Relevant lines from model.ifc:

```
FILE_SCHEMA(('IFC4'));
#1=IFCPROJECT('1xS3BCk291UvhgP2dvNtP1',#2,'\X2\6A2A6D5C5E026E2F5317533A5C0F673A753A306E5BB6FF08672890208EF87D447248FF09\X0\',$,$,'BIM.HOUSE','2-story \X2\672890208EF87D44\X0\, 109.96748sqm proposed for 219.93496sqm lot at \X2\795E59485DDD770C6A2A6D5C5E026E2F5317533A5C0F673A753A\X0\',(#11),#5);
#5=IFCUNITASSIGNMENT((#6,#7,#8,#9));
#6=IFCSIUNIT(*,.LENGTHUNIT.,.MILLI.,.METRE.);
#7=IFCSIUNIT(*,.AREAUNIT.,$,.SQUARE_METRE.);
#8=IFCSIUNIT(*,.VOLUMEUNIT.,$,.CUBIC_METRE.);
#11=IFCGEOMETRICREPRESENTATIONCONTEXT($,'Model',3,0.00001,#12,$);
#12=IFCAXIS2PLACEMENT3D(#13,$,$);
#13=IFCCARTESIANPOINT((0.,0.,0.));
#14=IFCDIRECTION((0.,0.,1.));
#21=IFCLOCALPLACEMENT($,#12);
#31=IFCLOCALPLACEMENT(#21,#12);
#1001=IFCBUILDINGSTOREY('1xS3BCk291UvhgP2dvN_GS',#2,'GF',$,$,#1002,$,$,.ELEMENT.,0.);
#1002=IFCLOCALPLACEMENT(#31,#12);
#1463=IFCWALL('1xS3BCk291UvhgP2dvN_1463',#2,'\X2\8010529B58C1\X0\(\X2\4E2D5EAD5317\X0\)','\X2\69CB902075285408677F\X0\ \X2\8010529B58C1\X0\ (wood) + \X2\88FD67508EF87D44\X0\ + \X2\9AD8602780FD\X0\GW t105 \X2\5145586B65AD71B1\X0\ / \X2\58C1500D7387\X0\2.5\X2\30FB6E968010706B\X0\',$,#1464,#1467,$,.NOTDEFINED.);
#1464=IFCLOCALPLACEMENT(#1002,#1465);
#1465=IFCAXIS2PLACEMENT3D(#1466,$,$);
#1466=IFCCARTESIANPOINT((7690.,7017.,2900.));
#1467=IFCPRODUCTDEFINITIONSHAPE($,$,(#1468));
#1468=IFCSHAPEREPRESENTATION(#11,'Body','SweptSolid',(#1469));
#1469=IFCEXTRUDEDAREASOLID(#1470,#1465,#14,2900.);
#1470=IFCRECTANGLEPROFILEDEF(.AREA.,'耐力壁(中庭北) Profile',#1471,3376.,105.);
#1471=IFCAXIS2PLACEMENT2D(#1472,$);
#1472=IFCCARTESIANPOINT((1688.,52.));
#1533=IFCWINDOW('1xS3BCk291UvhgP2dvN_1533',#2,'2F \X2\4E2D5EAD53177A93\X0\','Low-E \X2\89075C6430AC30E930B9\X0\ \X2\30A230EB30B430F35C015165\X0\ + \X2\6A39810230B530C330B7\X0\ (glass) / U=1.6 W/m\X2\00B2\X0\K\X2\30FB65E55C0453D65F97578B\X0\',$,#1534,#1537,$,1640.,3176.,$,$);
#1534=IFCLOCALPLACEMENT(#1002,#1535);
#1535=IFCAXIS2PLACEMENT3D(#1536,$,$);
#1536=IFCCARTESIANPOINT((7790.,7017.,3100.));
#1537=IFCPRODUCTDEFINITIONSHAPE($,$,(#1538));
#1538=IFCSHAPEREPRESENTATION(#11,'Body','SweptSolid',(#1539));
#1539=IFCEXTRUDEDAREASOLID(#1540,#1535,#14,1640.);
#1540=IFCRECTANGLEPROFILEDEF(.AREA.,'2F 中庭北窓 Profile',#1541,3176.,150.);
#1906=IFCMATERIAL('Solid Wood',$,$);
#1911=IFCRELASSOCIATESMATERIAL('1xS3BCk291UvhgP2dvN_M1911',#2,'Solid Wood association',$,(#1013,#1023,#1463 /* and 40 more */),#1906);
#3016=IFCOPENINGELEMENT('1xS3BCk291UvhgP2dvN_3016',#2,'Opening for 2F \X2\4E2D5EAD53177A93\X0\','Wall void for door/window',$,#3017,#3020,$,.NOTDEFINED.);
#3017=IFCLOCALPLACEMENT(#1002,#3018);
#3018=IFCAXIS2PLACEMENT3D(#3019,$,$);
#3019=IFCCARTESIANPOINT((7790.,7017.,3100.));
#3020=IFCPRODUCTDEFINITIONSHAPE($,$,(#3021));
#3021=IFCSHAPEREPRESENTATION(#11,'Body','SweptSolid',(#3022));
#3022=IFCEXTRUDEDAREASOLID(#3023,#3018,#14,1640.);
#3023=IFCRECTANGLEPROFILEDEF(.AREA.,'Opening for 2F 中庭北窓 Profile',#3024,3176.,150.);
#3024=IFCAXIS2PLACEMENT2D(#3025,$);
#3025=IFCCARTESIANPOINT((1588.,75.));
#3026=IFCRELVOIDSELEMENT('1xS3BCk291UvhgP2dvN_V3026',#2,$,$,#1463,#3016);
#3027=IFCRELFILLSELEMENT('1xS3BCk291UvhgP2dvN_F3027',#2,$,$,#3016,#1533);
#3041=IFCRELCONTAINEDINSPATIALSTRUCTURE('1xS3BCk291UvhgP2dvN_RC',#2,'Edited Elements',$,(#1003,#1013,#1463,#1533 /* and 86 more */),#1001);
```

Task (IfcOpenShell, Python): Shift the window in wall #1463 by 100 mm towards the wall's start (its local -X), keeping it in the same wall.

```python
import ifcopenshell
import ifcopenshell.api.geometry
import ifcopenshell.util.placement

model = ifcopenshell.open("model.ifc")

window = model.by_id(1533)
opening = window.FillsVoids[0].RelatingOpeningElement
wall = opening.VoidsElements[0].RelatingBuildingElement

wall_matrix = ifcopenshell.util.placement.get_local_placement(wall.ObjectPlacement)
shift = wall_matrix[:3, 0] * -100.0
before = ifcopenshell.util.placement.get_local_placement(window.ObjectPlacement)[:3, 3].copy()

# The window is not placed relative to its opening, so move both.
for product in (opening, window):
    matrix = ifcopenshell.util.placement.get_local_placement(product.ObjectPlacement)
    matrix[:3, 3] += shift
    ifcopenshell.api.geometry.edit_object_placement(model, product=product, matrix=matrix, is_si=False)

after = ifcopenshell.util.placement.get_local_placement(window.ObjectPlacement)[:3, 3]
print("window moved by", (after - before).round(3) + 0.0)

model.write("model_v2.ifc")
```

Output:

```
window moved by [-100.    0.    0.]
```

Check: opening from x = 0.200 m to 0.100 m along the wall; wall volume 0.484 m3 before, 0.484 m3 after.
